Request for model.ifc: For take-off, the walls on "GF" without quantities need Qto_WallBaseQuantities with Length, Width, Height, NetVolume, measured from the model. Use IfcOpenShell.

First a look at what the model holds.

```python
import ifcopenshell
import ifcopenshell.util.element
import ifcopenshell.util.unit

model = ifcopenshell.open("model.ifc")
print(model.schema)
for unit_type in ("LENGTHUNIT", "AREAUNIT", "VOLUMEUNIT"):
    print(unit_type, ifcopenshell.util.unit.calculate_unit_scale(model, unit_type))
storey = next(s for s in model.by_type("IfcBuildingStorey") if s.Name == "GF")
walls = [e for e in ifcopenshell.util.element.get_decomposition(storey) if e.is_a("IfcWall")]
for e in sorted(walls, key=lambda e: e.id()):
    print(e.id(), e.is_a(), e.Name, list(ifcopenshell.util.element.get_psets(e, qtos_only=True)), sep=" | ")
```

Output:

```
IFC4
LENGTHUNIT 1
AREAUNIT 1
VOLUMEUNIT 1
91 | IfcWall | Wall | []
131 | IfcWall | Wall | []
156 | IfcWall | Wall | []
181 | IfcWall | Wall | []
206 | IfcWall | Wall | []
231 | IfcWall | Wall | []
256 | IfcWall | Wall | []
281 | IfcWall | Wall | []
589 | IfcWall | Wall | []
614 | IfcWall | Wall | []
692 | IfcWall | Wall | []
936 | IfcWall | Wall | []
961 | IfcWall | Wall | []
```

```python
import ifcopenshell
import ifcopenshell.api.pset
import ifcopenshell.geom
import ifcopenshell.util.element
import ifcopenshell.util.shape
import ifcopenshell.util.unit

model = ifcopenshell.open("model.ifc")
unit_scale = ifcopenshell.util.unit.calculate_unit_scale(model)
volume_scale = ifcopenshell.util.unit.calculate_unit_scale(model, "VOLUMEUNIT")
settings = ifcopenshell.geom.settings()

storey = next(s for s in model.by_type("IfcBuildingStorey") if s.Name == "GF")
walls = [e for e in ifcopenshell.util.element.get_decomposition(storey) if e.is_a("IfcWall")]

for e in sorted(walls, key=lambda e: e.id()):
    if ifcopenshell.util.element.get_psets(e, qtos_only=True, should_inherit=False):
        continue
    # Geometry comes back in metres, in the element's own axes.
    shape = ifcopenshell.geom.create_shape(settings, e)
    values = {
        "Length": ifcopenshell.util.shape.get_x(shape.geometry) / unit_scale,
        "Width": ifcopenshell.util.shape.get_y(shape.geometry) / unit_scale,
        "Height": ifcopenshell.util.shape.get_z(shape.geometry) / unit_scale,
        "NetVolume": ifcopenshell.util.shape.get_volume(shape.geometry) / volume_scale,
    }
    qto = ifcopenshell.api.pset.add_qto(model, product=e, name="Qto_WallBaseQuantities")
    ifcopenshell.api.pset.edit_qto(model, qto=qto, properties=values)
    print(e.id(), {k: round(v, 3) for k, v in values.items()})

model.write("model_v2.ifc")
```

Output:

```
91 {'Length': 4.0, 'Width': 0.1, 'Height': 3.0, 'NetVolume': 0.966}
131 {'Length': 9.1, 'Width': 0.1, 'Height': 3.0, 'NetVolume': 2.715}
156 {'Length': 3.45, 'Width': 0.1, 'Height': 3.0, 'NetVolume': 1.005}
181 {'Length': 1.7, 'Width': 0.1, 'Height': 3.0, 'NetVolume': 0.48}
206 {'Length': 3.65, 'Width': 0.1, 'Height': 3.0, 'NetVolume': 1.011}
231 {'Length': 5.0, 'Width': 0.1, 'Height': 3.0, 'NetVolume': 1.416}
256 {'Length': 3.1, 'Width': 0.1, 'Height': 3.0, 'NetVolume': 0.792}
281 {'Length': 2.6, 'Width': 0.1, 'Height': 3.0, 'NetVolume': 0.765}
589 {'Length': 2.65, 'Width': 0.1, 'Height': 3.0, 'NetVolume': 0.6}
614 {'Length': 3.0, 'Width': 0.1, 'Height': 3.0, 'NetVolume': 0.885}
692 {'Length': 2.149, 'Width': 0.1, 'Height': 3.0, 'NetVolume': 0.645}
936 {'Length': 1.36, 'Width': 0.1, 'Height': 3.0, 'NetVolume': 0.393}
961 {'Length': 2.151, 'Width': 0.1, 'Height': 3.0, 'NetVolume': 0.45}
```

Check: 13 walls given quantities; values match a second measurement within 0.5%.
